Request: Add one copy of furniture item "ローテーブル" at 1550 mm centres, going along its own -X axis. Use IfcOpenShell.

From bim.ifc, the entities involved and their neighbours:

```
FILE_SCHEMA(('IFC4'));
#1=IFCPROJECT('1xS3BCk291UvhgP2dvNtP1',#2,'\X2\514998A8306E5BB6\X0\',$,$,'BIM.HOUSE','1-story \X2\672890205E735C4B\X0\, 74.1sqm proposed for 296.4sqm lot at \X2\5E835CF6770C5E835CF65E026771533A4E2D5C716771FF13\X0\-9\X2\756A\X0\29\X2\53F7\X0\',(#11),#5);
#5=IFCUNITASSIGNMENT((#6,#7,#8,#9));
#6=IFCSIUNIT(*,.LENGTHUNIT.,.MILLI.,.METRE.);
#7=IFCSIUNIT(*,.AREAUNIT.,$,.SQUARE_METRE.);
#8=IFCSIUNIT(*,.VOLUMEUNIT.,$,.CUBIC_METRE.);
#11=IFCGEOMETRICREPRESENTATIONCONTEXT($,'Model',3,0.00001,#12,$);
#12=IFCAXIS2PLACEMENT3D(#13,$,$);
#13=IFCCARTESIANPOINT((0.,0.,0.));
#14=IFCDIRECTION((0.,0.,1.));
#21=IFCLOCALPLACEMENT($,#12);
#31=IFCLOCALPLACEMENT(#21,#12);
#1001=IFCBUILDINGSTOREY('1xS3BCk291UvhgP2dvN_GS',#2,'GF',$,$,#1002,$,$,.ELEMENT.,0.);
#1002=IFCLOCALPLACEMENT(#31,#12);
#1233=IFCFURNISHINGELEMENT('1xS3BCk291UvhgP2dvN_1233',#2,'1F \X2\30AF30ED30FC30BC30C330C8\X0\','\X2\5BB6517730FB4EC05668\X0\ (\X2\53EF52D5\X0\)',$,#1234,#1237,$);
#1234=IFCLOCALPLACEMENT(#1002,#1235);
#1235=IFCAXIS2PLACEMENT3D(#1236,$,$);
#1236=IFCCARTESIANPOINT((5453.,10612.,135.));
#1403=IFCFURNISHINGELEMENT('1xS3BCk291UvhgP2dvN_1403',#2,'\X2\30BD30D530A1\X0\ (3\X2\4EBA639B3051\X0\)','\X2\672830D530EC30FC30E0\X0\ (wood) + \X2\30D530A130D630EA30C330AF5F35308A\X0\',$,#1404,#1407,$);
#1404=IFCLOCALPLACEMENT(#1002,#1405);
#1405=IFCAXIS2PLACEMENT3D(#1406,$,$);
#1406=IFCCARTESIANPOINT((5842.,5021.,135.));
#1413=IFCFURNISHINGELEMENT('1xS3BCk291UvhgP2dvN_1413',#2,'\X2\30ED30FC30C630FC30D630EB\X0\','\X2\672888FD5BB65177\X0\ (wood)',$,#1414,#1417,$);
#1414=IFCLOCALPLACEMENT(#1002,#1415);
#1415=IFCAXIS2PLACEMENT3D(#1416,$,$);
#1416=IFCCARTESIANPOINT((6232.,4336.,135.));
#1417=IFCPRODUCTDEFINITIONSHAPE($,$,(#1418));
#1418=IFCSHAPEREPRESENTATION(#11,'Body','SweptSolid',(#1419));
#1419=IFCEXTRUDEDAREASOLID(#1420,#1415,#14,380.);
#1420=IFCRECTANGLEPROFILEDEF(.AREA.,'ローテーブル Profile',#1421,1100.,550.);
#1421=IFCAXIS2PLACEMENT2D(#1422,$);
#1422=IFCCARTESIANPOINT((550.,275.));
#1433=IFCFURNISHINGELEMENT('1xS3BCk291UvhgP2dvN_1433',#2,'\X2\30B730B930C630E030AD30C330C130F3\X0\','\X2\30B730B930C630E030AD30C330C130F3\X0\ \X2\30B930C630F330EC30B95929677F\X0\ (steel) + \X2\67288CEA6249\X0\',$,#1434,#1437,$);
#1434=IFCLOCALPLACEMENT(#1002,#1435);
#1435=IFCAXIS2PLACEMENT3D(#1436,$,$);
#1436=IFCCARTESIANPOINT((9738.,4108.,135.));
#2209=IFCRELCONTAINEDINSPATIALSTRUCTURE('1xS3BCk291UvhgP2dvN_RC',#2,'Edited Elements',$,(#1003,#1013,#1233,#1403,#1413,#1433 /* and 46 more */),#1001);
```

```python
import ifcopenshell
import ifcopenshell.api.geometry
import ifcopenshell.api.root
import ifcopenshell.util.element
import ifcopenshell.util.placement
import ifcopenshell.util.unit

model = ifcopenshell.open("bim.ifc")
unit_scale = ifcopenshell.util.unit.calculate_unit_scale(model)


def reuse_history(source, copy):
    """copy_class also copies each property set's owner history, people and application; keep the originals."""
    for rel in copy.IsDefinedBy:
        if rel.is_a("IfcRelDefinesByProperties") and (history := rel.RelatingPropertyDefinition.OwnerHistory):
            rel.RelatingPropertyDefinition.OwnerHistory = source.OwnerHistory
            ifcopenshell.util.element.remove_deep2(model, history)


source = model.by_guid("1xS3BCk291UvhgP2dvN_1413")
base = ifcopenshell.util.placement.get_local_placement(source.ObjectPlacement)
step = -base[:3, 0] * 1.55 / unit_scale

for i in range(1, 2):
    copy = ifcopenshell.api.root.copy_class(model, product=source)
    copy.Representation = ifcopenshell.util.element.copy_deep(
        model, source.Representation, exclude=["IfcGeometricRepresentationContext", "IfcRepresentationMap"]
    )
    reuse_history(source, copy)
    matrix = base.copy()
    matrix[:3, 3] += i * step
    print("added at", matrix[:3, 3].round(3) + 0.0)
    ifcopenshell.api.geometry.edit_object_placement(model, product=copy, matrix=matrix, is_si=False)

model.write("bim-out.ifc")
```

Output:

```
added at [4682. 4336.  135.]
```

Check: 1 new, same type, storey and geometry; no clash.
